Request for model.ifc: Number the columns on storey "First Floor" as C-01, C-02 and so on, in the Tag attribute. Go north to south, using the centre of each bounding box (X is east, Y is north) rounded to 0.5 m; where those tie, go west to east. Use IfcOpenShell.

First a look at what the model holds.

```python
import ifcopenshell
import ifcopenshell.util.element
import ifcopenshell.util.placement

model = ifcopenshell.open("model.ifc")
print(model.schema)
storey = next(s for s in model.by_type("IfcBuildingStorey") if s.Name == "First Floor")
columns = [e for e in ifcopenshell.util.element.get_decomposition(storey) if e.is_a("IfcColumn")]
for e in sorted(columns, key=lambda e: e.id()):
    origin = ifcopenshell.util.placement.get_local_placement(e.ObjectPlacement)[:3, 3]
    print(e.id(), e.Tag, e.Name, origin.round(2) + 0.0, sep=" | ")
```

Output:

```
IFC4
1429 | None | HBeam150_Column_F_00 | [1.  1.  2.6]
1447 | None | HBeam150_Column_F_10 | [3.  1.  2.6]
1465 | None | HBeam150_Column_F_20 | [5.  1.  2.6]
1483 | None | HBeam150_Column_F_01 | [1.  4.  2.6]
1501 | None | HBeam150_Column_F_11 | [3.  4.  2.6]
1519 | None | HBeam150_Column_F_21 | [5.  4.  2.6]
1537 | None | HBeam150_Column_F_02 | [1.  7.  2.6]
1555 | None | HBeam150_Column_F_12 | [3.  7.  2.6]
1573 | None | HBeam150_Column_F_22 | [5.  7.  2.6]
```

```python
import ifcopenshell
import ifcopenshell.geom
import ifcopenshell.util.element
import ifcopenshell.util.shape

model = ifcopenshell.open("model.ifc")
settings = ifcopenshell.geom.settings()
settings.set("use-world-coords", True)


def centre(element):
    shape = ifcopenshell.geom.create_shape(settings, element)
    return ifcopenshell.util.shape.get_bbox_centroid(shape.geometry)


storey = next(s for s in model.by_type("IfcBuildingStorey") if s.Name == "First Floor")
columns = [e for e in ifcopenshell.util.element.get_decomposition(storey) if e.is_a("IfcColumn")]

# Insertion points can sit at a corner or the storey origin, so sort by the geometry (in metres).
centres = {e: centre(e) for e in columns}
columns.sort(key=lambda e: (-round(centres[e][1] / 0.5), centres[e][0]))

for i, e in enumerate(columns, start=1):
    number = f"C-{i:02d}"
    e.Tag = number
    print(e.id(), number)

model.write("model_edited.ifc")
```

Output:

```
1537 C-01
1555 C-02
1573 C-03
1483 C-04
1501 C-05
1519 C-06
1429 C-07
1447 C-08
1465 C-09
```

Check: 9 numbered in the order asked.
